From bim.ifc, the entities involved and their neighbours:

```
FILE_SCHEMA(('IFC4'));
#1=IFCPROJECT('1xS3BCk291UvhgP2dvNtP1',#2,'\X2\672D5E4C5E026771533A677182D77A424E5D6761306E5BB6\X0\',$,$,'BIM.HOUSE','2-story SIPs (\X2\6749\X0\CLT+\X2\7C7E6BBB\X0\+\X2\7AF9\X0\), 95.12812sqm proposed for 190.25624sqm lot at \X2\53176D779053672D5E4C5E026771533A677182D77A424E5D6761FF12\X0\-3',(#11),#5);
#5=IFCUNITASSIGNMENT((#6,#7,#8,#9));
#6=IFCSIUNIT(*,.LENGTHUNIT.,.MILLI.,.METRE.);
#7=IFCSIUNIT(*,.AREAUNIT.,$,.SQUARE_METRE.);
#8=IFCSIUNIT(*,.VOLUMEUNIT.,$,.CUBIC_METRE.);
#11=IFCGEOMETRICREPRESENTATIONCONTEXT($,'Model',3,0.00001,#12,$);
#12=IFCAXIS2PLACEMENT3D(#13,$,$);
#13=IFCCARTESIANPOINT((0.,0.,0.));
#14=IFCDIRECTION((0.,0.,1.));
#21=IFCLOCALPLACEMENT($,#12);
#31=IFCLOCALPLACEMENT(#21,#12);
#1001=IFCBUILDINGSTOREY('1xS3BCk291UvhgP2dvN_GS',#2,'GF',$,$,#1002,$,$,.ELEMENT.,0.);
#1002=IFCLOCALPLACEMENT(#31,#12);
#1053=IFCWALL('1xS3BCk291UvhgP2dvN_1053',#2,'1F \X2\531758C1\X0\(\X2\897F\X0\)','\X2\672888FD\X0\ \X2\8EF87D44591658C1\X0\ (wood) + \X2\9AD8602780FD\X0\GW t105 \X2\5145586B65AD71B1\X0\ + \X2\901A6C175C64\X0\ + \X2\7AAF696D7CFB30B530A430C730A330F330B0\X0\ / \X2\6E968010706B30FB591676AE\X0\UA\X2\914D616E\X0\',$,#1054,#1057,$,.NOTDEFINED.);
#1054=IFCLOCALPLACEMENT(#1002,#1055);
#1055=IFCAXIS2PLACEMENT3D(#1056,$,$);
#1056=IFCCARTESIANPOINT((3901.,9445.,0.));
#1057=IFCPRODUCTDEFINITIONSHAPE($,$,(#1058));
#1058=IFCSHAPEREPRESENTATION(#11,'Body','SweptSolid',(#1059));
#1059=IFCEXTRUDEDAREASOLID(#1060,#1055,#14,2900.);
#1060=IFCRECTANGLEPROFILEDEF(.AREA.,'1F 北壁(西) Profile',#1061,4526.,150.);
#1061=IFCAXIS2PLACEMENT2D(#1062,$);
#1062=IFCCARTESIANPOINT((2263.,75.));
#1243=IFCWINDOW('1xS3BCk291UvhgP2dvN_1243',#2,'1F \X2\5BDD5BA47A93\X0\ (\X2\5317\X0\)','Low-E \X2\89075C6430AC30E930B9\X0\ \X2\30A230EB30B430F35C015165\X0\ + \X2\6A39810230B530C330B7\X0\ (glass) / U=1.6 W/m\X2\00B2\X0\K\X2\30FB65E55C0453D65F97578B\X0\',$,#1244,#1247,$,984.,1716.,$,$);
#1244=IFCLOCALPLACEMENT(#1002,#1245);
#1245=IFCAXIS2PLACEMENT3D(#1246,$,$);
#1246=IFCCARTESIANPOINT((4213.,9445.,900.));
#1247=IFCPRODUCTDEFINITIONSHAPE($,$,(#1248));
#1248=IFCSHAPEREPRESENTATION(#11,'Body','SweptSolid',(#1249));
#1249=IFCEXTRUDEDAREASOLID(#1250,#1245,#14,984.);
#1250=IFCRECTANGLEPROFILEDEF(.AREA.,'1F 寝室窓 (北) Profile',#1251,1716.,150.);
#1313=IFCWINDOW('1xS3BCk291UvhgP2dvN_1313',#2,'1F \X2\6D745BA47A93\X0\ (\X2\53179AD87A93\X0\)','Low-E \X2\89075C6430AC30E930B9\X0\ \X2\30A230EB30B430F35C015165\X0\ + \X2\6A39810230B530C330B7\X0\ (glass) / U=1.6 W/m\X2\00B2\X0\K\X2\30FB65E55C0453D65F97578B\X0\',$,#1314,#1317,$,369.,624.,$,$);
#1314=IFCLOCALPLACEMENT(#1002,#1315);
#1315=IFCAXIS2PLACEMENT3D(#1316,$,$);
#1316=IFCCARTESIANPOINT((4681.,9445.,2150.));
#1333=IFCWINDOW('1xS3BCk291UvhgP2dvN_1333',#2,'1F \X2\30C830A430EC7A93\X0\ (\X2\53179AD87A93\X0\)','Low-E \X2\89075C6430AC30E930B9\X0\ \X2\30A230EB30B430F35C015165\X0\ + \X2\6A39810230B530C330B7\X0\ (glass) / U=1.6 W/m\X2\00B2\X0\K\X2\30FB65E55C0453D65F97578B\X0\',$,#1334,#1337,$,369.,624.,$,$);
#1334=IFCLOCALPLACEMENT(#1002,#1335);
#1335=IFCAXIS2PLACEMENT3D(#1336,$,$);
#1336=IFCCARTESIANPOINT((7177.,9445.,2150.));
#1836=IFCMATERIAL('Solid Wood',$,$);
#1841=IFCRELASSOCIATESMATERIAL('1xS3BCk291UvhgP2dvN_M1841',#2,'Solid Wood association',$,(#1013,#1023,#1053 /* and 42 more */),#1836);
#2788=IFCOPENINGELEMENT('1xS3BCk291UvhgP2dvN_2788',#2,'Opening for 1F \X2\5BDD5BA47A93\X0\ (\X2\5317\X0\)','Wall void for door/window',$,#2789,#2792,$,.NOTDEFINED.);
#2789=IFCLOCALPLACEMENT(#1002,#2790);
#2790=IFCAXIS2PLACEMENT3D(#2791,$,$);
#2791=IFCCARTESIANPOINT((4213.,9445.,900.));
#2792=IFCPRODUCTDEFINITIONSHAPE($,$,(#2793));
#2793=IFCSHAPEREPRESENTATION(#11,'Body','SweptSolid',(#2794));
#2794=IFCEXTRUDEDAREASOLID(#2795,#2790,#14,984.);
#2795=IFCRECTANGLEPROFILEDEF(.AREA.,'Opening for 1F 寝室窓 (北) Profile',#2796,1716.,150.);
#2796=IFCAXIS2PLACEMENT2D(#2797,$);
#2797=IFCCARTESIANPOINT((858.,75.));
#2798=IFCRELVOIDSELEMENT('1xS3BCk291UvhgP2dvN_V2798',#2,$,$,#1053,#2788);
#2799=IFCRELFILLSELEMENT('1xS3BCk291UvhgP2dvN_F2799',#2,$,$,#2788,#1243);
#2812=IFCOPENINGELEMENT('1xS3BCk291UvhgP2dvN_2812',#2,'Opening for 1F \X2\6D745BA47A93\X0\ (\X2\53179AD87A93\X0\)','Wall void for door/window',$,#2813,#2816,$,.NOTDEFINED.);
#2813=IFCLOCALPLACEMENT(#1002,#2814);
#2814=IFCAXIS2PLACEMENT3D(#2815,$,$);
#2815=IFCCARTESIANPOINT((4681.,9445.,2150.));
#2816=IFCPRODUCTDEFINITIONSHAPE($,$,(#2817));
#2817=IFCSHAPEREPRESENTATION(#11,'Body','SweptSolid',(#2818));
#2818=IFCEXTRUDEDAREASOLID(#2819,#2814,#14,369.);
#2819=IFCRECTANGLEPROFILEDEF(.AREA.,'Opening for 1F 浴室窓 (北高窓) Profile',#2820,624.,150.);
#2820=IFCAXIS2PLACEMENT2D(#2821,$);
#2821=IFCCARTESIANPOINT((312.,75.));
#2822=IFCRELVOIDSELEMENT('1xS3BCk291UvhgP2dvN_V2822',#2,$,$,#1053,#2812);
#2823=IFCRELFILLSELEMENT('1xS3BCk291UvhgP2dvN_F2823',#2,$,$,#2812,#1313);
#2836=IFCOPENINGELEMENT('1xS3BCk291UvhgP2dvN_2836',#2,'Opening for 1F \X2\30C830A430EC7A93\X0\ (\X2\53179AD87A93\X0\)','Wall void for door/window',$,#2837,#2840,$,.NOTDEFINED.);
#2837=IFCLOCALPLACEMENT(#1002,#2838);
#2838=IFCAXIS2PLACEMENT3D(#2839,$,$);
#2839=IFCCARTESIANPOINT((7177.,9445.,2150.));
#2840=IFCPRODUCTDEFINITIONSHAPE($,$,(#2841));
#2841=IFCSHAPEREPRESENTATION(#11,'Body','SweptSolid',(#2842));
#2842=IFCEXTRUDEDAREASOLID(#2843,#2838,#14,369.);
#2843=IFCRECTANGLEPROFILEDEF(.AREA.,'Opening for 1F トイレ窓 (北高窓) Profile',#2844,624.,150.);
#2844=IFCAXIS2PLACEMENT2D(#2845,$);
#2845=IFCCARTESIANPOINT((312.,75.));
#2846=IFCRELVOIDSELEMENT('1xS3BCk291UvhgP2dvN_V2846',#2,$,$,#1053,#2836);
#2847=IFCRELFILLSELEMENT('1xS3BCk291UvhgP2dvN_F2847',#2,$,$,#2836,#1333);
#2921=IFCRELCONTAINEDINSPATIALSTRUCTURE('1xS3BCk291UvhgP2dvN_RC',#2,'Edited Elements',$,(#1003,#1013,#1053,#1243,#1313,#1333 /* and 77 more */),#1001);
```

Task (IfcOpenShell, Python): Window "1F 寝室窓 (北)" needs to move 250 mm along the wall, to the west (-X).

```python
import ifcopenshell
import ifcopenshell.api.geometry
import ifcopenshell.util.placement

model = ifcopenshell.open("bim.ifc")

window = model.by_guid("1xS3BCk291UvhgP2dvN_1243")
opening = window.FillsVoids[0].RelatingOpeningElement
wall = opening.VoidsElements[0].RelatingBuildingElement

wall_matrix = ifcopenshell.util.placement.get_local_placement(wall.ObjectPlacement)
shift = wall_matrix[:3, 0] * -250.0
before = ifcopenshell.util.placement.get_local_placement(window.ObjectPlacement)[:3, 3].copy()

# The window is not placed relative to its opening, so move both.
for product in (opening, window):
    matrix = ifcopenshell.util.placement.get_local_placement(product.ObjectPlacement)
    matrix[:3, 3] += shift
    ifcopenshell.api.geometry.edit_object_placement(model, product=product, matrix=matrix, is_si=False)

after = ifcopenshell.util.placement.get_local_placement(window.ObjectPlacement)[:3, 3]
print("window moved by", (after - before).round(3) + 0.0)

model.write("bim_edited.ifc")
```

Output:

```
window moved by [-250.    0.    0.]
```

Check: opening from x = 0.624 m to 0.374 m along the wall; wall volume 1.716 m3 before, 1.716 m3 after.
